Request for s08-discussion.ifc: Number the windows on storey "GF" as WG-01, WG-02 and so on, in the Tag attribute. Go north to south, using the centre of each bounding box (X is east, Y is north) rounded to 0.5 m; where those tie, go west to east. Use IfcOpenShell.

First a look at what the model holds.

```python
import ifcopenshell
import ifcopenshell.util.element
import ifcopenshell.util.placement

model = ifcopenshell.open("s08-discussion.ifc")
print(model.schema)
storey = next(s for s in model.by_type("IfcBuildingStorey") if s.Name == "GF")
windows = [e for e in ifcopenshell.util.element.get_decomposition(storey) if e.is_a("IfcWindow")]
for e in sorted(windows, key=lambda e: e.id()):
    origin = ifcopenshell.util.placement.get_local_placement(e.ObjectPlacement)[:3, 3]
    print(e.id(), e.Tag, e.Name, origin.round(2) + 0.0, sep=" | ")
```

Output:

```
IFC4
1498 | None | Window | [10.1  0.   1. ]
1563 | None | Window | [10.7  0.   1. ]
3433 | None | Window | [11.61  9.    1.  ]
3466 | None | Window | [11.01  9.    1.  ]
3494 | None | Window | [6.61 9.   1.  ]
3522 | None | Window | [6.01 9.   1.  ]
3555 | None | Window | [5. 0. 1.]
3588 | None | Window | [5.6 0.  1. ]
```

```python
import ifcopenshell
import ifcopenshell.geom
import ifcopenshell.util.element
import ifcopenshell.util.shape

model = ifcopenshell.open("s08-discussion.ifc")
settings = ifcopenshell.geom.settings()
settings.set("use-world-coords", True)


def centre(element):
    shape = ifcopenshell.geom.create_shape(settings, element)
    return ifcopenshell.util.shape.get_bbox_centroid(shape.geometry)


storey = next(s for s in model.by_type("IfcBuildingStorey") if s.Name == "GF")
windows = [e for e in ifcopenshell.util.element.get_decomposition(storey) if e.is_a("IfcWindow")]

# Insertion points can sit at a corner or the storey origin, so sort by the geometry (in metres).
centres = {e: centre(e) for e in windows}
windows.sort(key=lambda e: (-round(centres[e][1] / 0.5), centres[e][0]))

for i, e in enumerate(windows, start=1):
    number = f"WG-{i:02d}"
    e.Tag = number
    print(e.id(), number)

model.write("s08-discussion_v2.ifc")
```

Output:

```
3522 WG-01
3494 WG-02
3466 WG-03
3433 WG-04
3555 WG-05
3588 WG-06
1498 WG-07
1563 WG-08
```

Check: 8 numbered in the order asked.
